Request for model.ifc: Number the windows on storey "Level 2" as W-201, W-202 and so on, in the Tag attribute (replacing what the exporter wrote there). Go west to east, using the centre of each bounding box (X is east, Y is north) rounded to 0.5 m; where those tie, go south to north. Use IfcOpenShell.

First a look at what the model holds.

```python
import ifcopenshell
import ifcopenshell.util.element
import ifcopenshell.util.placement

model = ifcopenshell.open("model.ifc")
print(model.schema)
storey = next(s for s in model.by_type("IfcBuildingStorey") if s.Name == "Level 2")
windows = [e for e in ifcopenshell.util.element.get_decomposition(storey) if e.is_a("IfcWindow")]
for e in sorted(windows, key=lambda e: e.id()):
    origin = ifcopenshell.util.placement.get_local_placement(e.ObjectPlacement)[:3, 3]
    print(e.id(), e.Tag, e.Name, origin.round(2) + 0.0, sep=" | ")
```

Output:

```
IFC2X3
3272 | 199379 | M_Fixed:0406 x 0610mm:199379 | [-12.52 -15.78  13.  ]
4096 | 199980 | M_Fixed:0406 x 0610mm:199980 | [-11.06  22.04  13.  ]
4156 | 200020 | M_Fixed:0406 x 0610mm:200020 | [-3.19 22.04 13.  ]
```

```python
import ifcopenshell
import ifcopenshell.geom
import ifcopenshell.util.element
import ifcopenshell.util.shape

model = ifcopenshell.open("model.ifc")
settings = ifcopenshell.geom.settings()
settings.set("use-world-coords", True)


def centre(element):
    shape = ifcopenshell.geom.create_shape(settings, element)
    return ifcopenshell.util.shape.get_bbox_centroid(shape.geometry)


storey = next(s for s in model.by_type("IfcBuildingStorey") if s.Name == "Level 2")
windows = [e for e in ifcopenshell.util.element.get_decomposition(storey) if e.is_a("IfcWindow")]

# Insertion points can sit at a corner or the storey origin, so sort by the geometry (in metres).
centres = {e: centre(e) for e in windows}
windows.sort(key=lambda e: (round(centres[e][0] / 0.5), centres[e][1]))

for i, e in enumerate(windows, start=1):
    number = f"W-2{i:02d}"
    e.Tag = number
    print(e.id(), number)

model.write("model_edited.ifc")
```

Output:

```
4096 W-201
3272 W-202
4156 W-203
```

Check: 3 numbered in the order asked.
